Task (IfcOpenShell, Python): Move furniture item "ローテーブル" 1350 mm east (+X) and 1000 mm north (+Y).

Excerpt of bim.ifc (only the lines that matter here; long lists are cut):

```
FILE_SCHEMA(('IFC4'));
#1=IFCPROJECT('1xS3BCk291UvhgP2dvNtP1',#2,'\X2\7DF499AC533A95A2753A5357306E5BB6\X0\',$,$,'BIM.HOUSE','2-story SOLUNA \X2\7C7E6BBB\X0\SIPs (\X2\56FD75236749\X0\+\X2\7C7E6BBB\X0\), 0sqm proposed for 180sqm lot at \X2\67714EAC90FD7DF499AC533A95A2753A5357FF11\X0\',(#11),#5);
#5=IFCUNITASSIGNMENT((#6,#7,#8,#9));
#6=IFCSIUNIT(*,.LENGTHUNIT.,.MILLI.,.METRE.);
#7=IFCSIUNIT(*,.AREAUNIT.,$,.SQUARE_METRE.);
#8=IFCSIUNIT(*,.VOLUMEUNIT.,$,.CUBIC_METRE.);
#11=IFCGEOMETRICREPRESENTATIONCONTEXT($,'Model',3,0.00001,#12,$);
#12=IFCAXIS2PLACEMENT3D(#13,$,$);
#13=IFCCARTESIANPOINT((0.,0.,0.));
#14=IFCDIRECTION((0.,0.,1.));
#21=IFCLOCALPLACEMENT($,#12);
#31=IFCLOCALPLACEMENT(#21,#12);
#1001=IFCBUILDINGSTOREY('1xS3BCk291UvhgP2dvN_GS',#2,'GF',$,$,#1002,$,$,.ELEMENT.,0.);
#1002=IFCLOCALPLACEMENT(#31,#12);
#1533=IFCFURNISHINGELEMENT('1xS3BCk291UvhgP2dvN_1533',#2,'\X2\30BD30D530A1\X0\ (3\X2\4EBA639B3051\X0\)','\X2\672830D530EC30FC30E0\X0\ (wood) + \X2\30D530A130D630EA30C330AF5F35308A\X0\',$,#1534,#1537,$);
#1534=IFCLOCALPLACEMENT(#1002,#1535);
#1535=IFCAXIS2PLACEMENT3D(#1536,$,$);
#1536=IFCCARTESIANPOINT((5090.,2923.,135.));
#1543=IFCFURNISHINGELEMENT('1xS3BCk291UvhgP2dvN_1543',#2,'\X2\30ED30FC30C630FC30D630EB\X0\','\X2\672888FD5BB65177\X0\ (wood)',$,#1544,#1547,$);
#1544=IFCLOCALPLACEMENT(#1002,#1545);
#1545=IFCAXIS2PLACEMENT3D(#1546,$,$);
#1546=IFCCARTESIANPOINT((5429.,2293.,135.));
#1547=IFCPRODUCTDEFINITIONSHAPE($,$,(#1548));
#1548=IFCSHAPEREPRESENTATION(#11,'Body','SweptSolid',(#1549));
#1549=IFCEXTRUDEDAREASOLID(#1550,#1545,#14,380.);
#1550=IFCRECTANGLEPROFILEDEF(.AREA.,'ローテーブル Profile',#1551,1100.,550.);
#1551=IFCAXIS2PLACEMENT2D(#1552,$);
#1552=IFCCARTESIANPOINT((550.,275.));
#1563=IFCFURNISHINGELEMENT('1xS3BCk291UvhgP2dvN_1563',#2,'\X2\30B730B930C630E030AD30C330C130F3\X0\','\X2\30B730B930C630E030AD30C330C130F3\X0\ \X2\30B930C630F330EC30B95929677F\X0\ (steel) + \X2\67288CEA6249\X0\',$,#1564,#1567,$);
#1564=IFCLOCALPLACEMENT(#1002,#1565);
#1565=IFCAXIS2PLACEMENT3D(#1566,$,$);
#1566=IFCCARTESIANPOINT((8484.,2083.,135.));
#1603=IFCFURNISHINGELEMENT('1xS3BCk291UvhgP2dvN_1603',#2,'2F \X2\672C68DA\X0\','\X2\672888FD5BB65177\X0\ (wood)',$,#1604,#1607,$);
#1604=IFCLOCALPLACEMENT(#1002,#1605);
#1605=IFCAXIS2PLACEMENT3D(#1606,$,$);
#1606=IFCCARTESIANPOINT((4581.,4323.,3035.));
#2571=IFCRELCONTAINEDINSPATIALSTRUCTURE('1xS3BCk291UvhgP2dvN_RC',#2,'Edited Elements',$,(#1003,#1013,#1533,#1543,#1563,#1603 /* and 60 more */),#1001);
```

```python
import ifcopenshell
import ifcopenshell.api.geometry
import ifcopenshell.util.placement

model = ifcopenshell.open("bim.ifc")

item = model.by_id(1543)
matrix = ifcopenshell.util.placement.get_local_placement(item.ObjectPlacement)
matrix[0, 3] += 1350.0
matrix[1, 3] += 1000.0
ifcopenshell.api.geometry.edit_object_placement(model, product=item, matrix=matrix, is_si=False)

print(ifcopenshell.util.placement.get_local_placement(item.ObjectPlacement).round(3) + 0.0)

model.write("bim-out.ifc")
```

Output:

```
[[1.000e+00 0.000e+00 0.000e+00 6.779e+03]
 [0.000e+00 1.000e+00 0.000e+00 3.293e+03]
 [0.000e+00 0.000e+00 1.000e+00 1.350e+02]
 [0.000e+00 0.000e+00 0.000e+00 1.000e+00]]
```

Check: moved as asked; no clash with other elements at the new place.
